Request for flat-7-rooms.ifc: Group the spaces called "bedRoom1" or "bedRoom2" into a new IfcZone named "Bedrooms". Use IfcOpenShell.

First a look at what the model holds.

```python
import ifcopenshell

model = ifcopenshell.open("flat-7-rooms.ifc")
print(model.schema)
seen = {}
for space in model.by_type("IfcSpace"):
    seen[space.LongName] = seen.get(space.LongName, 0) + 1
for name, count in sorted(seen.items(), key=str):
    print(count, "x", name)
print("zones:", [z.Name for z in model.by_type("IfcZone")][:20])
```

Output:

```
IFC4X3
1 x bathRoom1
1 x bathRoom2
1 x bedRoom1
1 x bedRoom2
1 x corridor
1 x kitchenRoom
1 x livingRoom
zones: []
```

```python
import ifcopenshell
import ifcopenshell.api.group
import ifcopenshell.api.root

model = ifcopenshell.open("flat-7-rooms.ifc")

names = {"bedRoom1", "bedRoom2"}
spaces = [s for s in model.by_type("IfcSpace") if s.LongName in names]

zone = ifcopenshell.api.root.create_entity(model, ifc_class="IfcZone", name="Bedrooms")
ifcopenshell.api.group.assign_group(model, products=spaces, group=zone)
print(len(spaces), "spaces in", zone.Name)

model.write("flat-7-rooms_updated.ifc")
```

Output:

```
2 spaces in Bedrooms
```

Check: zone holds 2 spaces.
